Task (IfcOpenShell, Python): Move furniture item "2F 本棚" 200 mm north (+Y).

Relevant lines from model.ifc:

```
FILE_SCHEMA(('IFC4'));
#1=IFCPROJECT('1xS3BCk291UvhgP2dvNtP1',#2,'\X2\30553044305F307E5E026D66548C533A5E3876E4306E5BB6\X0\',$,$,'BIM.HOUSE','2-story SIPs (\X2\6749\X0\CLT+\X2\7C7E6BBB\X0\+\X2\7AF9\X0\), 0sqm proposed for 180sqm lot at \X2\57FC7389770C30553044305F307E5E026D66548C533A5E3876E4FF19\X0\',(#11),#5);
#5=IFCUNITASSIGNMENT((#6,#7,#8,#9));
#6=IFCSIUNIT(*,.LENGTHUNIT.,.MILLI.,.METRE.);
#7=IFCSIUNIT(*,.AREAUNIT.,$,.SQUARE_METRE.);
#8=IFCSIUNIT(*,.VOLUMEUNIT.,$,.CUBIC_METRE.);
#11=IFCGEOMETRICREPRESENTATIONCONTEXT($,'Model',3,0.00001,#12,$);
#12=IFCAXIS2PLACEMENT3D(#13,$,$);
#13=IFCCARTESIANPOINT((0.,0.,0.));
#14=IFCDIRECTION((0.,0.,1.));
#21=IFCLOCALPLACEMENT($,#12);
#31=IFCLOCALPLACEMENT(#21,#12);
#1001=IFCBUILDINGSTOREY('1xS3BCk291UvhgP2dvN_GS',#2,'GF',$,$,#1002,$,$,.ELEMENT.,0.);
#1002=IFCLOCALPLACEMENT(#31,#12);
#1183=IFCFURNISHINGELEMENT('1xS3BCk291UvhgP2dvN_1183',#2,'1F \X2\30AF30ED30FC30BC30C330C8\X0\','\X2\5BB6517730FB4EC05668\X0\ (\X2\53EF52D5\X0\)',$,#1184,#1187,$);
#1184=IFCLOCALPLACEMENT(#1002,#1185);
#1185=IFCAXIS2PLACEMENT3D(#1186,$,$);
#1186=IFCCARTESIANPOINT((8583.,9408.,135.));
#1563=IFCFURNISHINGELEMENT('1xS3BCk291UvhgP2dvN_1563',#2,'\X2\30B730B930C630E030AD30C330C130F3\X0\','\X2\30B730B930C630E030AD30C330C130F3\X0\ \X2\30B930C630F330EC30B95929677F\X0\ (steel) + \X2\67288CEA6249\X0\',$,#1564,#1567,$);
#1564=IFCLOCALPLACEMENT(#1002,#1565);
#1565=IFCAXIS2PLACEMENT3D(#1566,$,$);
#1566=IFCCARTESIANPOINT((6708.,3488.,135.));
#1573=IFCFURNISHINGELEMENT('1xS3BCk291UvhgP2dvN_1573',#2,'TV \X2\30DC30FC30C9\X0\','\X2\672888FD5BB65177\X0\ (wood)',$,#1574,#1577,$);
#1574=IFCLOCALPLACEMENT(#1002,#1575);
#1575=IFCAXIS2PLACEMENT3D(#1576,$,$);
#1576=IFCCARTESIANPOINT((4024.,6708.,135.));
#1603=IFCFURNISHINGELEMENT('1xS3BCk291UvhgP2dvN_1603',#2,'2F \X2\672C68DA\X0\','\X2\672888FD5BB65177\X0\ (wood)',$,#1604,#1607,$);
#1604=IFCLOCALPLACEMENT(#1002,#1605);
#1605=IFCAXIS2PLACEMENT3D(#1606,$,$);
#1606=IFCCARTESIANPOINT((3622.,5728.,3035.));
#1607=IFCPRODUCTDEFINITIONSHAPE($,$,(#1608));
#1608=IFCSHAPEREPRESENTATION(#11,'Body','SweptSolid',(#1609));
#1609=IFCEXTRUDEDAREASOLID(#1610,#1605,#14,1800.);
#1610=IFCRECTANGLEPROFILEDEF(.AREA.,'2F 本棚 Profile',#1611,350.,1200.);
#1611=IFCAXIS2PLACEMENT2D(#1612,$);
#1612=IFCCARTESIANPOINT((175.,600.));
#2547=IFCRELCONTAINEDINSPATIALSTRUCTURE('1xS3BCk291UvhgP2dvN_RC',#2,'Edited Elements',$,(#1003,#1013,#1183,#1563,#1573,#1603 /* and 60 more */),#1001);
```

```python
import ifcopenshell
import ifcopenshell.api.geometry
import ifcopenshell.util.placement
import ifcopenshell.util.unit

model = ifcopenshell.open("model.ifc")
unit_scale = ifcopenshell.util.unit.calculate_unit_scale(model)

item = model.by_guid("1xS3BCk291UvhgP2dvN_1603")
matrix = ifcopenshell.util.placement.get_local_placement(item.ObjectPlacement)
matrix[1, 3] += 0.2 / unit_scale
ifcopenshell.api.geometry.edit_object_placement(model, product=item, matrix=matrix, is_si=False)

print(ifcopenshell.util.placement.get_local_placement(item.ObjectPlacement).round(3) + 0.0)

model.write("model_edited.ifc")
```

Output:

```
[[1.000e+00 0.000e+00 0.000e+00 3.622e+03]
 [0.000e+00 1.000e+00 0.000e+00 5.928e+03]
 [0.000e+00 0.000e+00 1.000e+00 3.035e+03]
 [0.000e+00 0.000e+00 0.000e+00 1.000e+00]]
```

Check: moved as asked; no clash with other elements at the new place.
